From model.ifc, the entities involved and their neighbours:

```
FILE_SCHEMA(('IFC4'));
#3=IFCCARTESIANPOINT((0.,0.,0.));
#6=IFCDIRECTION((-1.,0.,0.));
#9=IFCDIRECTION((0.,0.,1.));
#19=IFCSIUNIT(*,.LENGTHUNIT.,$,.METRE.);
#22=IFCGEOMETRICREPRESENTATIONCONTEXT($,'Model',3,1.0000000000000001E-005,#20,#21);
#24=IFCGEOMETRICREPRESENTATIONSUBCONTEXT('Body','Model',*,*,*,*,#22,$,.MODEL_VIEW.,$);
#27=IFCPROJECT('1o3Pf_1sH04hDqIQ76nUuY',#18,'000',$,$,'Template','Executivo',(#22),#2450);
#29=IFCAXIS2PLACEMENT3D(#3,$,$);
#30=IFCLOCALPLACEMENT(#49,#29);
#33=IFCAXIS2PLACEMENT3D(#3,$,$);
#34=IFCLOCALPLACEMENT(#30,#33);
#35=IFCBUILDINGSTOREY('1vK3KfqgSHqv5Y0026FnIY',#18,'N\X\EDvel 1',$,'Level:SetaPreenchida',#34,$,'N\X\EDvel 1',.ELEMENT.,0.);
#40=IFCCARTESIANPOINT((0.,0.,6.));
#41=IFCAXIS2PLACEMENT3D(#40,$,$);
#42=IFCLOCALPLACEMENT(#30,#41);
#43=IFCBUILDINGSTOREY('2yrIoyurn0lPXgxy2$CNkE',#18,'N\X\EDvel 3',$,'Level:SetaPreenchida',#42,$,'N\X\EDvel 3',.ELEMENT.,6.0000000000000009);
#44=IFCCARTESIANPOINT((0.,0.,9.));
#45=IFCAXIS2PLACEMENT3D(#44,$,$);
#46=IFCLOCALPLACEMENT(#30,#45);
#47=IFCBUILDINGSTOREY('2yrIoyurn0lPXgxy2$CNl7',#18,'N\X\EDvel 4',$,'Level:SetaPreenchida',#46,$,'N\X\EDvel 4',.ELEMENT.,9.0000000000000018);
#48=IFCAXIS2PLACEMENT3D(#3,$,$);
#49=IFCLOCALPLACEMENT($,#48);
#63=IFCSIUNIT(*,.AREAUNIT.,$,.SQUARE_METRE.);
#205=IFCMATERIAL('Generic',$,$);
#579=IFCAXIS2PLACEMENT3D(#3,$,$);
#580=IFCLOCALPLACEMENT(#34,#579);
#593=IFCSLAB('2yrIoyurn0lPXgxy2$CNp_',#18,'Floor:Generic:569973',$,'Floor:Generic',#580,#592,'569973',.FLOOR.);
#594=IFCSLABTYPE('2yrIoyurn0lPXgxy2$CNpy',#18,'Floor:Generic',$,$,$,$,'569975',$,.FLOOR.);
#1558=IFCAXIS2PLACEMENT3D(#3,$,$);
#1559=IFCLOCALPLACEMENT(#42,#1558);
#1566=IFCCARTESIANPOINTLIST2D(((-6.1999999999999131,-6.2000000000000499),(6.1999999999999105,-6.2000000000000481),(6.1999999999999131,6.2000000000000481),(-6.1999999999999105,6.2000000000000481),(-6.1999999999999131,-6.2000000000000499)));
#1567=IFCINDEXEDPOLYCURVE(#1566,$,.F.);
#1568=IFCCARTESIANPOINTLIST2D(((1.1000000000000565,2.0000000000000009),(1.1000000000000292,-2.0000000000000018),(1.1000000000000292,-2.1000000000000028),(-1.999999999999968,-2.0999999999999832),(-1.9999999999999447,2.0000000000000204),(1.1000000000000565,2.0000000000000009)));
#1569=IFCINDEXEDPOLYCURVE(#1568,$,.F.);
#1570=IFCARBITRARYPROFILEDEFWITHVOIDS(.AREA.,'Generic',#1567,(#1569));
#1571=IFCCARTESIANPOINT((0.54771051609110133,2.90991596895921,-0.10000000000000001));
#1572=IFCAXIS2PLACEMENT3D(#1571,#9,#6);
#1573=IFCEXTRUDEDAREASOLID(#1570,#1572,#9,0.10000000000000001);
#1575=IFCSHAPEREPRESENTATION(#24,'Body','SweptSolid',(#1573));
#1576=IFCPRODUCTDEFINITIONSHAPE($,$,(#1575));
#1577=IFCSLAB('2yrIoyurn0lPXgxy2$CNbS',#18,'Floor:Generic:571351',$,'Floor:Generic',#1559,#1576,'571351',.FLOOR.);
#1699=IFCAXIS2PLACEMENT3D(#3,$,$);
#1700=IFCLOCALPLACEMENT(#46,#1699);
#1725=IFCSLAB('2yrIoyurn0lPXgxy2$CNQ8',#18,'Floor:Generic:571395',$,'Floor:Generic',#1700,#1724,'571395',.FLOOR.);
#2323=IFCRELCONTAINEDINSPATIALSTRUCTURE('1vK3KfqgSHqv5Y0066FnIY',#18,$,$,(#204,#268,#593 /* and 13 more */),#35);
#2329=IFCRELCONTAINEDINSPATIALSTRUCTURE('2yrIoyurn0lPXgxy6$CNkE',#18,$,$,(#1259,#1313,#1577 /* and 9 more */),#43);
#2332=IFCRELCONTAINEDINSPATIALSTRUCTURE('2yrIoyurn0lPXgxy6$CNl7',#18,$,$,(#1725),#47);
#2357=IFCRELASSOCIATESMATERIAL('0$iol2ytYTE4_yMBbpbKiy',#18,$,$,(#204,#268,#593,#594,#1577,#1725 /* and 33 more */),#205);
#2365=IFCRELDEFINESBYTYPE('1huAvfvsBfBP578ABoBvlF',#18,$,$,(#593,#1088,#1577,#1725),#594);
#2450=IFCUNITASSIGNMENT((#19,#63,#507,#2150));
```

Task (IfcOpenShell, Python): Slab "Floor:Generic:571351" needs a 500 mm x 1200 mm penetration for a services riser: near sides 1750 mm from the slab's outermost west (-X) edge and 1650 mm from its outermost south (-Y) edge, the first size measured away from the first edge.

```python
import numpy as np
import ifcopenshell
import ifcopenshell.api.feature
import ifcopenshell.api.geometry
import ifcopenshell.api.root
import ifcopenshell.geom
import ifcopenshell.util.placement
import ifcopenshell.util.representation
import ifcopenshell.util.shape
import ifcopenshell.util.unit

model = ifcopenshell.open("model.ifc")
unit_scale = ifcopenshell.util.unit.calculate_unit_scale(model)
settings = ifcopenshell.geom.settings()


def volume(element):
    """Net volume in cubic metres, openings subtracted."""
    shape = ifcopenshell.geom.create_shape(settings, element)
    return ifcopenshell.util.shape.get_volume(shape.geometry)


slab = model.by_guid("2yrIoyurn0lPXgxy2$CNbS")
before = volume(slab)

# Extent in the slab's own axes, in metres. The edges named are its -X and -Y sides.
slab_shape = ifcopenshell.geom.create_shape(settings, slab)
vertices = ifcopenshell.util.shape.get_vertices(slab_shape.geometry)
x_min, y_min, bottom = vertices.min(axis=0)
top = vertices[:, 2].max()

opening = ifcopenshell.api.root.create_entity(model, ifc_class="IfcOpeningElement", name="Services riser opening", predefined_type="OPENING")
context = ifcopenshell.util.representation.get_context(model, "Model", "Body", "MODEL_VIEW")
width, depth = 0.5, 1.2
outline = [(0.0, 0.0), (width, 0.0), (width, depth), (0.0, depth), (0.0, 0.0)]
# Overshoot both faces by 50 mm so the cut is clean.
shape = ifcopenshell.api.geometry.add_slab_representation(
    model, context=context, depth=top - bottom + 0.1, polyline=outline
)
ifcopenshell.api.geometry.assign_representation(model, product=opening, representation=shape)

matrix = ifcopenshell.util.placement.get_local_placement(slab.ObjectPlacement)
matrix[:, 3] = matrix @ np.append(np.array([x_min + 1.75, y_min + 1.65, bottom - 0.05]) / unit_scale, 1.0)
ifcopenshell.api.geometry.edit_object_placement(model, product=opening, matrix=matrix, is_si=False)
ifcopenshell.api.feature.add_feature(model, feature=opening, element=slab)

after = volume(slab)

print(f"slab volume {before:.3f} -> {after:.3f} m3")

model.write("model_updated.ifc")
```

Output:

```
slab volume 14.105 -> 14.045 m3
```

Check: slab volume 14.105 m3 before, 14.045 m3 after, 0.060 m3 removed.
